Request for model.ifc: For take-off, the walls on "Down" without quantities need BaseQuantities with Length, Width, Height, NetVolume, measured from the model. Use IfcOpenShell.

First a look at what the model holds.

```python
import ifcopenshell
import ifcopenshell.util.element
import ifcopenshell.util.unit

model = ifcopenshell.open("model.ifc")
print(model.schema)
for unit_type in ("LENGTHUNIT", "AREAUNIT", "VOLUMEUNIT"):
    print(unit_type, ifcopenshell.util.unit.calculate_unit_scale(model, unit_type))
storey = next(s for s in model.by_type("IfcBuildingStorey") if s.Name == "Down")
walls = [e for e in ifcopenshell.util.element.get_decomposition(storey) if e.is_a("IfcWall")]
for e in sorted(walls, key=lambda e: e.id()):
    print(e.id(), e.is_a(), e.Name, list(ifcopenshell.util.element.get_psets(e, qtos_only=True)), sep=" | ")
```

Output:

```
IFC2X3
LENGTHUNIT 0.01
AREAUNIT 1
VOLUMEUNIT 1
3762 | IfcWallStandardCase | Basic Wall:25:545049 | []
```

```python
import ifcopenshell
import ifcopenshell.api.pset
import ifcopenshell.geom
import ifcopenshell.util.element
import ifcopenshell.util.shape
import ifcopenshell.util.unit

model = ifcopenshell.open("model.ifc")
unit_scale = ifcopenshell.util.unit.calculate_unit_scale(model)
volume_scale = ifcopenshell.util.unit.calculate_unit_scale(model, "VOLUMEUNIT")
settings = ifcopenshell.geom.settings()

storey = next(s for s in model.by_type("IfcBuildingStorey") if s.Name == "Down")
walls = [e for e in ifcopenshell.util.element.get_decomposition(storey) if e.is_a("IfcWall")]

for e in sorted(walls, key=lambda e: e.id()):
    if ifcopenshell.util.element.get_psets(e, qtos_only=True, should_inherit=False):
        continue
    # Geometry comes back in metres, in the element's own axes.
    shape = ifcopenshell.geom.create_shape(settings, e)
    values = {
        "Length": ifcopenshell.util.shape.get_x(shape.geometry) / unit_scale,
        "Width": ifcopenshell.util.shape.get_y(shape.geometry) / unit_scale,
        "Height": ifcopenshell.util.shape.get_z(shape.geometry) / unit_scale,
        "NetVolume": ifcopenshell.util.shape.get_volume(shape.geometry) / volume_scale,
    }
    qto = ifcopenshell.api.pset.add_qto(model, product=e, name="BaseQuantities")
    ifcopenshell.api.pset.edit_qto(model, qto=qto, properties=values)
    print(e.id(), {k: round(v, 3) for k, v in values.items()})

model.write("model_rev.ifc")
```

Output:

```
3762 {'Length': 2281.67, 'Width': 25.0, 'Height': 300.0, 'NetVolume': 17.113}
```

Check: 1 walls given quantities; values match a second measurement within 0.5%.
